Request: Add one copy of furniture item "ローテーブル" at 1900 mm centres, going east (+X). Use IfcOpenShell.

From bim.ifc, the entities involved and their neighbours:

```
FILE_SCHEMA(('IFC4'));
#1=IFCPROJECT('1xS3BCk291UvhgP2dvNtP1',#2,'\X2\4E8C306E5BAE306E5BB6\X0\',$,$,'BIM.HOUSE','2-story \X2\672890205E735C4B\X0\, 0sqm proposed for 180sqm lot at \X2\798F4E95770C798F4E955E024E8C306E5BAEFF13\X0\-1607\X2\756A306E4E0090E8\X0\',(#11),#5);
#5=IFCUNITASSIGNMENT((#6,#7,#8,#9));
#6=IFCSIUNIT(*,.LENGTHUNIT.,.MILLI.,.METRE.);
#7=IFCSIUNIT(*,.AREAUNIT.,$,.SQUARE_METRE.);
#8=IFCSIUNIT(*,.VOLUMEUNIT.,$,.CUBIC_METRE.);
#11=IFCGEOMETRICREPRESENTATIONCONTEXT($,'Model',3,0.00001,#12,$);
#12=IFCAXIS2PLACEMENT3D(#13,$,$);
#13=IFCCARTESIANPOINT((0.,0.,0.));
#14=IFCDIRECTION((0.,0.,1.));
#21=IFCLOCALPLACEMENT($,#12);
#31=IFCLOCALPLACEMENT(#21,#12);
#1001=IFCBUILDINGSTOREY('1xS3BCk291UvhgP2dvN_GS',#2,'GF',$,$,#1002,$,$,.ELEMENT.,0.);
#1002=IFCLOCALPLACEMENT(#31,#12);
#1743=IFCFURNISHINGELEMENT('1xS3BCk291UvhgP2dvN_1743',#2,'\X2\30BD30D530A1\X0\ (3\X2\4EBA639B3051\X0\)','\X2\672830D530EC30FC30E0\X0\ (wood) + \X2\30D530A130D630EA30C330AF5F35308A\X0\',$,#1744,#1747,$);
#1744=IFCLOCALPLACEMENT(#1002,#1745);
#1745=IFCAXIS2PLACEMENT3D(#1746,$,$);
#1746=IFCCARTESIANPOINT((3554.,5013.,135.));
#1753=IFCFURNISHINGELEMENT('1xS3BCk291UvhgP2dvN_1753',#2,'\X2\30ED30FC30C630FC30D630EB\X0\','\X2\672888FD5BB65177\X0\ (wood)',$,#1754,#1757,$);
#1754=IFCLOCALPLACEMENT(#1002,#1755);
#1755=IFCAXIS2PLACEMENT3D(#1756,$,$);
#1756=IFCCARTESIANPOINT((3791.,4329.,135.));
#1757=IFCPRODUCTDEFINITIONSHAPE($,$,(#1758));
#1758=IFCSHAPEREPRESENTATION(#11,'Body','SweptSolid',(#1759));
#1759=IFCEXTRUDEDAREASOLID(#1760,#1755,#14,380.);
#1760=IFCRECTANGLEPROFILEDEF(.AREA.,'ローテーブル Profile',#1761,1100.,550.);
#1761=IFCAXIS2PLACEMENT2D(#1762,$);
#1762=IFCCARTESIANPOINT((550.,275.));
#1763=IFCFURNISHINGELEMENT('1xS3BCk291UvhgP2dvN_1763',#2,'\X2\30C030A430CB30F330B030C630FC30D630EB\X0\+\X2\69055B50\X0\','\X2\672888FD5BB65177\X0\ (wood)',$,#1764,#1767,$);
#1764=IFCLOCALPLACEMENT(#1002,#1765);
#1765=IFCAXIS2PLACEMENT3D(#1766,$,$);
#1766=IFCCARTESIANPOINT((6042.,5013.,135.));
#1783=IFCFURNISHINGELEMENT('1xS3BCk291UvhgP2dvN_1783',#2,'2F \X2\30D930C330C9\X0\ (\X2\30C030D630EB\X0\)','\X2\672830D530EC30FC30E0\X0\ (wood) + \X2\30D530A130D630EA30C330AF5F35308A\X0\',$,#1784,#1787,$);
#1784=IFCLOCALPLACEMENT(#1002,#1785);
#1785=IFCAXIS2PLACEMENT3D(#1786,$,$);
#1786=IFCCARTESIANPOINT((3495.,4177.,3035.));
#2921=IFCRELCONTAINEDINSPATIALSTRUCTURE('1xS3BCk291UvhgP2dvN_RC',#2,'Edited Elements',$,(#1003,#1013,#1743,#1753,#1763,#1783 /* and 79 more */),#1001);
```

```python
import numpy as np
import ifcopenshell
import ifcopenshell.api.geometry
import ifcopenshell.api.root
import ifcopenshell.util.element
import ifcopenshell.util.placement
import ifcopenshell.util.unit

model = ifcopenshell.open("bim.ifc")
unit_scale = ifcopenshell.util.unit.calculate_unit_scale(model)


def reuse_history(source, copy):
    """copy_class also copies each property set's owner history, people and application; keep the originals."""
    for rel in copy.IsDefinedBy:
        if rel.is_a("IfcRelDefinesByProperties") and (history := rel.RelatingPropertyDefinition.OwnerHistory):
            rel.RelatingPropertyDefinition.OwnerHistory = source.OwnerHistory
            ifcopenshell.util.element.remove_deep2(model, history)


source = model.by_id(1753)
base = ifcopenshell.util.placement.get_local_placement(source.ObjectPlacement)
step = np.array([1.0, 0.0, 0.0]) * 1.9 / unit_scale

for i in range(1, 2):
    copy = ifcopenshell.api.root.copy_class(model, product=source)
    copy.Representation = ifcopenshell.util.element.copy_deep(
        model, source.Representation, exclude=["IfcGeometricRepresentationContext", "IfcRepresentationMap"]
    )
    reuse_history(source, copy)
    matrix = base.copy()
    matrix[:3, 3] += i * step
    print("added at", matrix[:3, 3].round(3) + 0.0)
    ifcopenshell.api.geometry.edit_object_placement(model, product=copy, matrix=matrix, is_si=False)

model.write("bim_v2.ifc")
```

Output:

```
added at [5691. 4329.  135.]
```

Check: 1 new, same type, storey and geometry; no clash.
